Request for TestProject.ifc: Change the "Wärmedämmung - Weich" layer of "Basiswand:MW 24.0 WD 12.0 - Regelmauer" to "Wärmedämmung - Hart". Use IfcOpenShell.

First a look at what the model holds.

```python
import ifcopenshell
import ifcopenshell.util.element

model = ifcopenshell.open("TestProject.ifc")
print(model.schema)
for layer_set in model.by_type("IfcMaterialLayerSet"):
    if layer_set.LayerSetName == "Basiswand:MW 24.0 WD 12.0 - Regelmauer":
        for layer in layer_set.MaterialLayers:
            print(layer.id(), layer.Material and layer.Material.Name, layer.LayerThickness, sep=" | ")
        print(len(ifcopenshell.util.element.get_elements_by_material(model, layer_set)), "elements and types use it")
print(sorted(m.Name for m in model.by_type("IfcMaterial") if m.Name)[:60])
```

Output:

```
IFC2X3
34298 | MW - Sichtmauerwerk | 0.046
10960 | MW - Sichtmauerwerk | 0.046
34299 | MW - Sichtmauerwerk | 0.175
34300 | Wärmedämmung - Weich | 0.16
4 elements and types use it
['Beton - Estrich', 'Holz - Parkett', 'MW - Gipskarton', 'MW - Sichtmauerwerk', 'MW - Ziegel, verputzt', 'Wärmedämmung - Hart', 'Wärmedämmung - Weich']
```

```python
import ifcopenshell
import ifcopenshell.api.material

model = ifcopenshell.open("TestProject.ifc")

layer_set = next(s for s in model.by_type("IfcMaterialLayerSet") if s.LayerSetName == "Basiswand:MW 24.0 WD 12.0 - Regelmauer")
layer = next(l for l in layer_set.MaterialLayers if l.Material and l.Material.Name == "Wärmedämmung - Weich")
material = next(m for m in model.by_type("IfcMaterial") if m.Name == "Wärmedämmung - Hart")

# Point this one layer at the other material; renaming the old one would change it everywhere.
ifcopenshell.api.material.edit_layer(model, layer=layer, attributes={}, material=material)

print([l.Material.Name if l.Material else None for l in layer_set.MaterialLayers])

model.write("TestProject_v2.ifc")
```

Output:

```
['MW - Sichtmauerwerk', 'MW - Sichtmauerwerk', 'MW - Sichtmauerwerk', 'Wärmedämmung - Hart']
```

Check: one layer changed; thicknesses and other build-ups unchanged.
